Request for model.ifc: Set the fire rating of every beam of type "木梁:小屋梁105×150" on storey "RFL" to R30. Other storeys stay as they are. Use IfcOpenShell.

First a look at what the model holds.

```python
import ifcopenshell
import ifcopenshell.util.element

model = ifcopenshell.open("model.ifc")
print(model.schema)
storey = next(s for s in model.by_type("IfcBuildingStorey") if s.Name == "RFL")
beams = [e for e in ifcopenshell.util.element.get_decomposition(storey) if e.is_a("IfcBeam")]
seen = {}
for e in beams:
    element_type = ifcopenshell.util.element.get_type(e)
    key = (element_type.Name if element_type != e and element_type else None, ifcopenshell.util.element.get_pset(e, "Pset_BeamCommon", "FireRating"))
    seen[key] = seen.get(key, 0) + 1
for (name, value), count in sorted(seen.items(), key=str):
    print(count, "x", name, "|", value)
```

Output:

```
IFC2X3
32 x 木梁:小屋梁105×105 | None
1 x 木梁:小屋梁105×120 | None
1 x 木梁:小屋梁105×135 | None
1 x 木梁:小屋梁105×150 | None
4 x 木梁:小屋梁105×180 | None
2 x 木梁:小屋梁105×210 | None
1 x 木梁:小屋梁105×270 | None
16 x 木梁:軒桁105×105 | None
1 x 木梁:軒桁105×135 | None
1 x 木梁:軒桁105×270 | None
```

```python
import ifcopenshell
import ifcopenshell.api.pset
import ifcopenshell.util.element

model = ifcopenshell.open("model.ifc")

storey = next(s for s in model.by_type("IfcBuildingStorey") if s.Name == "RFL")
beams = [e for e in ifcopenshell.util.element.get_decomposition(storey) if e.is_a("IfcBeam")]

count = 0
for e in beams:
    element_type = ifcopenshell.util.element.get_type(e)
    if element_type in (None, e) or element_type.Name != "木梁:小屋梁105×150":
        continue
    # add_pset returns the element's existing set when there is one.
    pset = ifcopenshell.api.pset.add_pset(model, product=e, name="Pset_BeamCommon")
    ifcopenshell.api.pset.edit_pset(model, pset=pset, properties={"FireRating": "R30"})
    count += 1

print(count, "beams updated")

model.write("model_rev.ifc")
```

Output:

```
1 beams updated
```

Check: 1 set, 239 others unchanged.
